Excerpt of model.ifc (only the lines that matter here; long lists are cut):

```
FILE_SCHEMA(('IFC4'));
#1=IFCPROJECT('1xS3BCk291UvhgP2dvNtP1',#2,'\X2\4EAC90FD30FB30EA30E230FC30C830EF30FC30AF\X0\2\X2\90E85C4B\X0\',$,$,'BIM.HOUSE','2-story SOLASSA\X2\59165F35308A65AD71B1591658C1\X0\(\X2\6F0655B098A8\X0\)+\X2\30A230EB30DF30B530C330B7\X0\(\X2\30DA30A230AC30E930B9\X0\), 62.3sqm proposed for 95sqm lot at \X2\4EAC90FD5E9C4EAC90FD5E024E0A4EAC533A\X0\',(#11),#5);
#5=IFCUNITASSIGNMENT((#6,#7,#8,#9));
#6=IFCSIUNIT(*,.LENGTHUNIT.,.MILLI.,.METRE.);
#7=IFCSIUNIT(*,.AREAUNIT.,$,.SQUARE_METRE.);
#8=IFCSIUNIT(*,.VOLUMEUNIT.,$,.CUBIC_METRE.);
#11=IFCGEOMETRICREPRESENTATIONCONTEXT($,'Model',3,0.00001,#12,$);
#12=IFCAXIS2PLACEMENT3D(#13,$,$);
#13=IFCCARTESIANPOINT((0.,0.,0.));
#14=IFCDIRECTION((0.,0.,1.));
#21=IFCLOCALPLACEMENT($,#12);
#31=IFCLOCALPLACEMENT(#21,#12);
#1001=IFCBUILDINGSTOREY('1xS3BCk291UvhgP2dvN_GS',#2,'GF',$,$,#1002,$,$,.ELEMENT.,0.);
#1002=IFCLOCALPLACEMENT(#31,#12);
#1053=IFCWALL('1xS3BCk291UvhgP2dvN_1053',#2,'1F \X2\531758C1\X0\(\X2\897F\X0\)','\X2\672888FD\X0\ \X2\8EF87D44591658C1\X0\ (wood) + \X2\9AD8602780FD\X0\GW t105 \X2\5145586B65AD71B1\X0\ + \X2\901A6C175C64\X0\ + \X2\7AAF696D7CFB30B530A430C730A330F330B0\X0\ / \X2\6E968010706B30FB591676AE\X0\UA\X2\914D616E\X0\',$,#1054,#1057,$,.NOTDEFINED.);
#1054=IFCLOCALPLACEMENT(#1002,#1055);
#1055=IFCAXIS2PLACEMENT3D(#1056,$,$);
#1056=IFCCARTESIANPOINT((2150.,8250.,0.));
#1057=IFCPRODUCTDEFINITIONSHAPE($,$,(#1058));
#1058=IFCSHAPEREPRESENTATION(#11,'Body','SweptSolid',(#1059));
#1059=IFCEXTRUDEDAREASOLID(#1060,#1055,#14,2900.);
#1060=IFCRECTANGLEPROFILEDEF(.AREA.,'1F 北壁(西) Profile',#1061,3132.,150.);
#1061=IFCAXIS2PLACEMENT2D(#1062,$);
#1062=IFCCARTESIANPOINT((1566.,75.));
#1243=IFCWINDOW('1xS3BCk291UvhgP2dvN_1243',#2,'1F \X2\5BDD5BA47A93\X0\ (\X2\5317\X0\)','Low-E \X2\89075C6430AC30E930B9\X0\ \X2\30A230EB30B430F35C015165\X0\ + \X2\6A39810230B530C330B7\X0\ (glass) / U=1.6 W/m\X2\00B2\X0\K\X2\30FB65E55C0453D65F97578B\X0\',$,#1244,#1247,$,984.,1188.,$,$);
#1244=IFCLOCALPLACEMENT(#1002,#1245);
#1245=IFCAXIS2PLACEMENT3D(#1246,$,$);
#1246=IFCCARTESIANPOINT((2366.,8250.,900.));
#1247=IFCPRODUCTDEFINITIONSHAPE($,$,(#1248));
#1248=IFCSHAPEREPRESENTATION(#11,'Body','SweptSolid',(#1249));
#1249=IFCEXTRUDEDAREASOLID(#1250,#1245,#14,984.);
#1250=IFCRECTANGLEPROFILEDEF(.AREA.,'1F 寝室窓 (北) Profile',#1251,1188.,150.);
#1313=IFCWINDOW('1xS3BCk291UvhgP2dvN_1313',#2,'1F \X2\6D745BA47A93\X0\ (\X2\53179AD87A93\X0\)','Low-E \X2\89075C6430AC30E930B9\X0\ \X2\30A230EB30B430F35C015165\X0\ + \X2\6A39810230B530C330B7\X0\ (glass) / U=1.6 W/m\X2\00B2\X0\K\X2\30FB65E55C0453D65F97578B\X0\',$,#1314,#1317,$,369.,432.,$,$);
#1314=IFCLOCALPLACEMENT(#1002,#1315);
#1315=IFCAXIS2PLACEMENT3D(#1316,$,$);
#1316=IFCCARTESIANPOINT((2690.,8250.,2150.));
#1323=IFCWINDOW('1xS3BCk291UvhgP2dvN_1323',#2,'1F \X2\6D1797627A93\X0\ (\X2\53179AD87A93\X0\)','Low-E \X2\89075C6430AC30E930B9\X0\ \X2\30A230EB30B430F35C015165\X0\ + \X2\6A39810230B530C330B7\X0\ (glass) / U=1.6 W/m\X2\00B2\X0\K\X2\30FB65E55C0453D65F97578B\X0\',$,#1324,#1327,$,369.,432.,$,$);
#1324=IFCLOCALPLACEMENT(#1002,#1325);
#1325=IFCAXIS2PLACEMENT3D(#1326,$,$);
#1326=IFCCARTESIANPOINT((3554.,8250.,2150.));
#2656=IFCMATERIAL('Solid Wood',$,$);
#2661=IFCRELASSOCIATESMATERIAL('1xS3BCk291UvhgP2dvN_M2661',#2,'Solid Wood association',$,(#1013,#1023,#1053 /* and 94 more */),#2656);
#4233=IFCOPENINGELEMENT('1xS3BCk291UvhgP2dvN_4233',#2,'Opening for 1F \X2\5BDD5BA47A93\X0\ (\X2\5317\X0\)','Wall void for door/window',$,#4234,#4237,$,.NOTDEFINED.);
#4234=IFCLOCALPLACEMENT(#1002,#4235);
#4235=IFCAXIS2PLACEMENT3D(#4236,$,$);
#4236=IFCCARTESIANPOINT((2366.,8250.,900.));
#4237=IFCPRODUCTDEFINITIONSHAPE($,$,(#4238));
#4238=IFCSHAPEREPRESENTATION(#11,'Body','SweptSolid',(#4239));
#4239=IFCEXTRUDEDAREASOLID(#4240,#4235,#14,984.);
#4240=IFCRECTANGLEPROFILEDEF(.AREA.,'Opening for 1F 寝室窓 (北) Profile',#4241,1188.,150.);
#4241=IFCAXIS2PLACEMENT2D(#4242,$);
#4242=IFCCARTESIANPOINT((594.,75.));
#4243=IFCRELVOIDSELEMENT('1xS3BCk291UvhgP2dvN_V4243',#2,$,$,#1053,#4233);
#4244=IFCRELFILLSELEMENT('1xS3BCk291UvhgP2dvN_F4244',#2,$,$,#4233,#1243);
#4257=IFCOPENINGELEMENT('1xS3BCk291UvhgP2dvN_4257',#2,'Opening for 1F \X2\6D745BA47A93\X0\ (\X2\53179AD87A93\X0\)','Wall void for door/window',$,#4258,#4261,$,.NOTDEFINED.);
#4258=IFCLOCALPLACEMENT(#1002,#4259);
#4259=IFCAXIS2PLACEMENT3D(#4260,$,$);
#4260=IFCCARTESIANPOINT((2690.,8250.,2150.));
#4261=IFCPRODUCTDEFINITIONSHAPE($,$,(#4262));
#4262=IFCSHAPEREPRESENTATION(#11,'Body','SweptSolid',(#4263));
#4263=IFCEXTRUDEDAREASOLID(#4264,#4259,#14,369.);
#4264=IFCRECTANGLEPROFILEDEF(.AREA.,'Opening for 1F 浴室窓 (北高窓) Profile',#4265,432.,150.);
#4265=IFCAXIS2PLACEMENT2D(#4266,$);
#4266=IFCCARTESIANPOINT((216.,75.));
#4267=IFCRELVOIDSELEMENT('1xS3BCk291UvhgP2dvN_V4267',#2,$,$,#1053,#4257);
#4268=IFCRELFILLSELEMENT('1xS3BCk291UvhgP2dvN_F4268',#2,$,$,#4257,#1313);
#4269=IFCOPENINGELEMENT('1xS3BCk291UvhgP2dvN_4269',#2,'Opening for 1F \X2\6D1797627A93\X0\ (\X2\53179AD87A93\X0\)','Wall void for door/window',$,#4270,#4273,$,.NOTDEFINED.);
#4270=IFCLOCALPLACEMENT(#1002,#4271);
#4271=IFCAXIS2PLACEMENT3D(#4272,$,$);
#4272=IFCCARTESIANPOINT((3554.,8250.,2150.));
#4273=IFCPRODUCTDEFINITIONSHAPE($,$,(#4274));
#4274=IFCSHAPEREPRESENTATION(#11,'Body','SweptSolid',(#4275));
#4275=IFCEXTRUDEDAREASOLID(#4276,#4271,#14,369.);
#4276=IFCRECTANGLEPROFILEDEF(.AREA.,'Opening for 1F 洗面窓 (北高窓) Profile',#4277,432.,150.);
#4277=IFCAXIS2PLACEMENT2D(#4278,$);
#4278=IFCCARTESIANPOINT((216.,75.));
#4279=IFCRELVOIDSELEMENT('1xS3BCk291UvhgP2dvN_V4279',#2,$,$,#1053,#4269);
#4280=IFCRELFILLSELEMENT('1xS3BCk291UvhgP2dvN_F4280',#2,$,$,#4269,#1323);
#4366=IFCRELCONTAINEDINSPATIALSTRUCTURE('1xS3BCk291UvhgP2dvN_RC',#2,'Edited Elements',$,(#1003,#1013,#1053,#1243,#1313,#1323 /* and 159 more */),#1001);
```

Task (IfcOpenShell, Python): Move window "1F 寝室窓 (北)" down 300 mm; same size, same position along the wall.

```python
import numpy as np
import ifcopenshell
import ifcopenshell.api.geometry
import ifcopenshell.util.placement
import ifcopenshell.util.unit

model = ifcopenshell.open("model.ifc")
unit_scale = ifcopenshell.util.unit.calculate_unit_scale(model)

window = model.by_guid("1xS3BCk291UvhgP2dvN_1243")
opening = window.FillsVoids[0].RelatingOpeningElement
dz = -0.3 / unit_scale

shift = np.array([0.0, 0.0, dz])
# The window is not placed relative to its opening, so move both.
for product in (opening, window):
    matrix = ifcopenshell.util.placement.get_local_placement(product.ObjectPlacement)
    matrix[:3, 3] += shift
    ifcopenshell.api.geometry.edit_object_placement(model, product=product, matrix=matrix, is_si=False)

print(f"moved by {dz * unit_scale:+.3f} m")

model.write("model_updated.ifc")
```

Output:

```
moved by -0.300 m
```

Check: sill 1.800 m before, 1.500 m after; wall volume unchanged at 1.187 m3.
